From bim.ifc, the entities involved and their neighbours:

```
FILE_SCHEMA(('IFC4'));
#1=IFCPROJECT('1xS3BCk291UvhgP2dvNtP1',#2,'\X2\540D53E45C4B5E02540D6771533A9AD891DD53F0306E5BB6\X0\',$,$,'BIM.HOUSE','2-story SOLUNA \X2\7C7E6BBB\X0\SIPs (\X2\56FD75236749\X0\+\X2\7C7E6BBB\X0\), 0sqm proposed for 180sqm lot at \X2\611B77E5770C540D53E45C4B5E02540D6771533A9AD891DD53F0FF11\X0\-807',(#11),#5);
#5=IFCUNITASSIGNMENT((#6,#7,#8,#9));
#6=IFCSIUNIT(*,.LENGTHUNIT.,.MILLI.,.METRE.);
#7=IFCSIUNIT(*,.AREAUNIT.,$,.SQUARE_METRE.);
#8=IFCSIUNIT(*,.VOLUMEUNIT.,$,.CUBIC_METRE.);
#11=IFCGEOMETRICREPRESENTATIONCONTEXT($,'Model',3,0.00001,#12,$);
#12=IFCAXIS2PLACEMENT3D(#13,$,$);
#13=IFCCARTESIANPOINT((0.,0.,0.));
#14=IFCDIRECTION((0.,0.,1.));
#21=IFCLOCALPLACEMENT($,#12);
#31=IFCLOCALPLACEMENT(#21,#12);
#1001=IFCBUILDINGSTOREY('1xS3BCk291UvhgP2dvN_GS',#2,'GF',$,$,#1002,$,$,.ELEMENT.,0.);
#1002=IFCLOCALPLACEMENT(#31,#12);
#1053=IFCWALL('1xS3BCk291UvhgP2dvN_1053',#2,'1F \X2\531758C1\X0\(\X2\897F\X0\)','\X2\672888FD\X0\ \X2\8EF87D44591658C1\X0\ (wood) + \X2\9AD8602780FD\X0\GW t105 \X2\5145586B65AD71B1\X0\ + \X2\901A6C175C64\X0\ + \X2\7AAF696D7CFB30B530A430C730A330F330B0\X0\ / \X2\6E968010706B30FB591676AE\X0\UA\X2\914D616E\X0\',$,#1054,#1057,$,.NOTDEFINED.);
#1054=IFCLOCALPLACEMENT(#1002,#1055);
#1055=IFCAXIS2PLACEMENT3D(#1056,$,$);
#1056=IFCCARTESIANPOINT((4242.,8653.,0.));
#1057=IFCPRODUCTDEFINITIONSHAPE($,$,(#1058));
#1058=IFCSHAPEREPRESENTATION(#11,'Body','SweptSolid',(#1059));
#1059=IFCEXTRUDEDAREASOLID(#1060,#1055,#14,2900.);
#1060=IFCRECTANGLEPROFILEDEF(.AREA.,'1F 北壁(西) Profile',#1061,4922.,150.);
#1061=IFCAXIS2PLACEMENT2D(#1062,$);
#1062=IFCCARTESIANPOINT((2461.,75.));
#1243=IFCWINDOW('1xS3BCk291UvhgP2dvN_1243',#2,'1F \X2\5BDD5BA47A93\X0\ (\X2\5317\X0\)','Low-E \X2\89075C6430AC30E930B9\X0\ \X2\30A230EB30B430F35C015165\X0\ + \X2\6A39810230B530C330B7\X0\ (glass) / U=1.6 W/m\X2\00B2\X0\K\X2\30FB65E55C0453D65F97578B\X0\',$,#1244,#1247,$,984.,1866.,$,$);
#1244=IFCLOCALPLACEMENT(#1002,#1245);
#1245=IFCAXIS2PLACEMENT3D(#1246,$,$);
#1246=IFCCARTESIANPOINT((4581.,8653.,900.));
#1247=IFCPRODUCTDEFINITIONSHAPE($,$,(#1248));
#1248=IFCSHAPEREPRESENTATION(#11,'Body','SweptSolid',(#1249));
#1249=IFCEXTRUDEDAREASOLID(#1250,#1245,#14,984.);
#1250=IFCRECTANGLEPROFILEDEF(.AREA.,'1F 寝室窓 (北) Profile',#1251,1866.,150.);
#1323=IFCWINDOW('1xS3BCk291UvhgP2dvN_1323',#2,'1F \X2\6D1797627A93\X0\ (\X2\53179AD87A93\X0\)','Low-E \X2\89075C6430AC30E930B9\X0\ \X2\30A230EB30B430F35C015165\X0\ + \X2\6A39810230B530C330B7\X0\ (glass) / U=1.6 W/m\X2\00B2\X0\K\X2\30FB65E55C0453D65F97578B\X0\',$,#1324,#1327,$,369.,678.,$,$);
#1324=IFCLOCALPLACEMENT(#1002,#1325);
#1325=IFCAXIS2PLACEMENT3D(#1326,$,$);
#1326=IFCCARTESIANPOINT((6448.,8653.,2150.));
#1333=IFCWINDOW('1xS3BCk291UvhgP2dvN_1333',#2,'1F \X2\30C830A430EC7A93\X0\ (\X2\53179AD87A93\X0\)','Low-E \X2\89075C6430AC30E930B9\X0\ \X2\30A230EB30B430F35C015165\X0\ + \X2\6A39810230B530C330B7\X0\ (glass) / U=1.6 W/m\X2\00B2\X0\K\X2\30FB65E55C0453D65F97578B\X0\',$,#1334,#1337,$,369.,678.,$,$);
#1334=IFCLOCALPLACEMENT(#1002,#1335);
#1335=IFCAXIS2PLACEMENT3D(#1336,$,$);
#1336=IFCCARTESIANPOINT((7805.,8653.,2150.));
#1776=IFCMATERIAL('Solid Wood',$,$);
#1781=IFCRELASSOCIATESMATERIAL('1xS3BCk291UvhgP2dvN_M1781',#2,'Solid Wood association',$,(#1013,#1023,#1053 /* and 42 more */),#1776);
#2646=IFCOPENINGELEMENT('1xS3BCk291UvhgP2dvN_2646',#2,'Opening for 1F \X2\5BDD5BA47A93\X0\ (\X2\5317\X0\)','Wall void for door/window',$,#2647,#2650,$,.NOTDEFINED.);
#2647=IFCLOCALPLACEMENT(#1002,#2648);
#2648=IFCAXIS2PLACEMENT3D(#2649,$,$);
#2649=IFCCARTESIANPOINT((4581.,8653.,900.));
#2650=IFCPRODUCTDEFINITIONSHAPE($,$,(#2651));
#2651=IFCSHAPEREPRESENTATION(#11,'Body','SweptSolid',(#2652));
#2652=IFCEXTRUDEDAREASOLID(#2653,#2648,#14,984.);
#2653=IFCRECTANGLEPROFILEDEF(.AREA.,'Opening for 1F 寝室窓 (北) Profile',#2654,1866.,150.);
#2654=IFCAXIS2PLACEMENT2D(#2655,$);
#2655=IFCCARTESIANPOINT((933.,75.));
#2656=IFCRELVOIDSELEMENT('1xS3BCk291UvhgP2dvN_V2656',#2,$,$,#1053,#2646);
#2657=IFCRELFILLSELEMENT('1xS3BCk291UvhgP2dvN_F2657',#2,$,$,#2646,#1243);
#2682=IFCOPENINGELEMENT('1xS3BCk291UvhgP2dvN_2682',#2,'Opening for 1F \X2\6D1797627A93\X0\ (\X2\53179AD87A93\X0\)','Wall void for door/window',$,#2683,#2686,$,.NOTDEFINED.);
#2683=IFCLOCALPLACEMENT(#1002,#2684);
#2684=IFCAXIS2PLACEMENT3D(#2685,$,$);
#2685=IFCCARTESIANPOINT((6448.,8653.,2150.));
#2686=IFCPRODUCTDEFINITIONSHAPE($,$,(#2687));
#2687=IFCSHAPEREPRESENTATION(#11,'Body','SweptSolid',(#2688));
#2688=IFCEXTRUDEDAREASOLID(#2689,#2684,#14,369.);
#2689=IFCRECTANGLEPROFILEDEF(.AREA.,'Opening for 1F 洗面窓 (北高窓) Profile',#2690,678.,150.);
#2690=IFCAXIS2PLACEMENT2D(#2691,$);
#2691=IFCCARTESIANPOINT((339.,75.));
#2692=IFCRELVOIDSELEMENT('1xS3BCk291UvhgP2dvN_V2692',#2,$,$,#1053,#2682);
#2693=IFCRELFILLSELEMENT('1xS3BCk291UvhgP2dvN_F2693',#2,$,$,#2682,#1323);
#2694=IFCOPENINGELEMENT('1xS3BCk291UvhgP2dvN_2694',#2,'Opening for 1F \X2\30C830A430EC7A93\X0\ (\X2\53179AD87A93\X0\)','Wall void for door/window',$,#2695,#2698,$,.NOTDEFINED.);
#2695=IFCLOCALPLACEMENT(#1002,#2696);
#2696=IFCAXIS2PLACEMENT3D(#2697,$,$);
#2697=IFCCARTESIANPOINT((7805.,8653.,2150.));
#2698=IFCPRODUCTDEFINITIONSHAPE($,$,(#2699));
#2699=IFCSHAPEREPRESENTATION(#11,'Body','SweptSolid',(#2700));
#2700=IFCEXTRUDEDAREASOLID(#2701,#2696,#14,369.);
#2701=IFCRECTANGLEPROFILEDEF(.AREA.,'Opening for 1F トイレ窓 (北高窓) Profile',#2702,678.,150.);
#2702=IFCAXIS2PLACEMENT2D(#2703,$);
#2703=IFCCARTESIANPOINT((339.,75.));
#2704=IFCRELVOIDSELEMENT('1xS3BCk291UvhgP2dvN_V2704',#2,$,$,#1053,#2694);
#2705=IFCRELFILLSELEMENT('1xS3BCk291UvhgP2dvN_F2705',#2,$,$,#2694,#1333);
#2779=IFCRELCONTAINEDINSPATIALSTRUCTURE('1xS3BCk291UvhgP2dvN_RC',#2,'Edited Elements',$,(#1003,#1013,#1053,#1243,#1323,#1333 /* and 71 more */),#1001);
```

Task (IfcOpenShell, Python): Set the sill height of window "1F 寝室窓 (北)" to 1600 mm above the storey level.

```python
import numpy as np
import ifcopenshell
import ifcopenshell.api.geometry
import ifcopenshell.geom
import ifcopenshell.util.element
import ifcopenshell.util.placement
import ifcopenshell.util.shape
import ifcopenshell.util.unit

model = ifcopenshell.open("bim.ifc")
unit_scale = ifcopenshell.util.unit.calculate_unit_scale(model)

window = model.by_guid("1xS3BCk291UvhgP2dvN_1243")
opening = window.FillsVoids[0].RelatingOpeningElement
storey = ifcopenshell.util.element.get_container(window, ifc_class="IfcBuildingStorey")
level = ifcopenshell.util.placement.get_local_placement(storey.ObjectPlacement)[2, 3]

# The opening's origin need not be at the sill, so measure its lowest point.
shape = ifcopenshell.geom.create_shape(ifcopenshell.geom.settings(), opening)
bottom = ifcopenshell.util.shape.get_shape_bottom_elevation(shape, shape.geometry) / unit_scale
dz = level + 1.6 / unit_scale - bottom

shift = np.array([0.0, 0.0, dz])
# The window is not placed relative to its opening, so move both.
for product in (opening, window):
    matrix = ifcopenshell.util.placement.get_local_placement(product.ObjectPlacement)
    matrix[:3, 3] += shift
    ifcopenshell.api.geometry.edit_object_placement(model, product=product, matrix=matrix, is_si=False)

print(f"moved by {dz * unit_scale:+.3f} m")

model.write("bim_v2.ifc")
```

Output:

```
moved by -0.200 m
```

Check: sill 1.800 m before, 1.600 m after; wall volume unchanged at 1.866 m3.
